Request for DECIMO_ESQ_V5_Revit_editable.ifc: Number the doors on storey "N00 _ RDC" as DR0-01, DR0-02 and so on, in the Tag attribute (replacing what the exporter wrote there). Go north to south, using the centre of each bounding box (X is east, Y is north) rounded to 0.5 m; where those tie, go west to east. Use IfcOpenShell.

First a look at what the model holds.

```python
import ifcopenshell
import ifcopenshell.util.element
import ifcopenshell.util.placement

model = ifcopenshell.open("DECIMO_ESQ_V5_Revit_editable.ifc")
print(model.schema)
storey = next(s for s in model.by_type("IfcBuildingStorey") if s.Name == "N00 _ RDC")
doors = [e for e in ifcopenshell.util.element.get_decomposition(storey) if e.is_a("IfcDoor")]
for e in sorted(doors, key=lambda e: e.id()):
    origin = ifcopenshell.util.placement.get_local_placement(e.ObjectPlacement)[:3, 3]
    print(e.id(), e.Tag, e.Name, origin.round(2) + 0.0, sep=" | ")
```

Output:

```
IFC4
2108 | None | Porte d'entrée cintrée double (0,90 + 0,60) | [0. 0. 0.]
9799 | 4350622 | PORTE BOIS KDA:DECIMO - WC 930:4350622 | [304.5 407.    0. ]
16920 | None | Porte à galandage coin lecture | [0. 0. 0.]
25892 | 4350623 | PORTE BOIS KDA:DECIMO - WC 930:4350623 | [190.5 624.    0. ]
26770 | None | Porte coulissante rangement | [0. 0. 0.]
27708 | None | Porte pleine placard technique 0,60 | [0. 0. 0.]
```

```python
import ifcopenshell
import ifcopenshell.geom
import ifcopenshell.util.element
import ifcopenshell.util.shape

model = ifcopenshell.open("DECIMO_ESQ_V5_Revit_editable.ifc")
settings = ifcopenshell.geom.settings()
settings.set("use-world-coords", True)


def centre(element):
    shape = ifcopenshell.geom.create_shape(settings, element)
    return ifcopenshell.util.shape.get_bbox_centroid(shape.geometry)


storey = next(s for s in model.by_type("IfcBuildingStorey") if s.Name == "N00 _ RDC")
doors = [e for e in ifcopenshell.util.element.get_decomposition(storey) if e.is_a("IfcDoor")]

# Insertion points can sit at a corner or the storey origin, so sort by the geometry (in metres).
centres = {e: centre(e) for e in doors}
doors.sort(key=lambda e: (-round(centres[e][1] / 0.5), centres[e][0]))

for i, e in enumerate(doors, start=1):
    number = f"DR0-{i:02d}"
    e.Tag = number
    print(e.id(), number)

model.write("DECIMO_ESQ_V5_Revit_editable_edited.ifc")
```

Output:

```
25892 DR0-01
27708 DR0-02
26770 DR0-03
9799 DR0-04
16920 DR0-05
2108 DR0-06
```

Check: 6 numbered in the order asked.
